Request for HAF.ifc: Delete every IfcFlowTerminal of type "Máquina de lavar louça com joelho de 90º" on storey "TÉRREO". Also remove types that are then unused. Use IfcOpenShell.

First a look at what the model holds.

```python
import ifcopenshell
import ifcopenshell.util.element

model = ifcopenshell.open("HAF.ifc")
print(model.schema)
storey = next(s for s in model.by_type("IfcBuildingStorey") if s.Name == "TÉRREO")
terminals = [e for e in ifcopenshell.util.element.get_decomposition(storey) if e.is_a("IfcFlowTerminal")]
seen = {}
for e in terminals:
    element_type = ifcopenshell.util.element.get_type(e)
    name = element_type.Name if element_type not in (None, e) else None
    seen[name] = seen.get(name, 0) + 1
for name, count in sorted(seen.items(), key=str):
    print(count, "x", name)
```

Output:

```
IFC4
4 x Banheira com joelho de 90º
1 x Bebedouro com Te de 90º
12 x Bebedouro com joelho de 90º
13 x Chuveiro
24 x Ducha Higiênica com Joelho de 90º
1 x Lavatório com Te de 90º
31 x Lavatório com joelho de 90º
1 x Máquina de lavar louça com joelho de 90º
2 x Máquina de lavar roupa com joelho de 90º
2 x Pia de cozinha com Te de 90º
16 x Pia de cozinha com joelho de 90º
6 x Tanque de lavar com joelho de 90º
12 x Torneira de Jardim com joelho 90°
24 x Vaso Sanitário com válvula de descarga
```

```python
import ifcopenshell
import ifcopenshell.api.root
import ifcopenshell.util.element

model = ifcopenshell.open("HAF.ifc")

storey = next(s for s in model.by_type("IfcBuildingStorey") if s.Name == "TÉRREO")
terminals = [e for e in ifcopenshell.util.element.get_decomposition(storey) if e.is_a("IfcFlowTerminal")]
targets = [e for e in terminals if (t := ifcopenshell.util.element.get_type(e)) not in (None, e) and t.Name == "Máquina de lavar louça com joelho de 90º"]
types = {ifcopenshell.util.element.get_type(e) for e in targets} - {None, *targets}

for e in targets:
    ifcopenshell.api.root.remove_product(model, product=e)
print(len(targets), "removed")

unused = [t for t in types if not ifcopenshell.util.element.get_types(t)]
for t in unused:
    ifcopenshell.api.root.remove_product(model, product=t)
print(len(unused), "unused types removed")

model.write("HAF_edited.ifc")
```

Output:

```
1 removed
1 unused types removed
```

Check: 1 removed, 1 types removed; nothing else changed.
